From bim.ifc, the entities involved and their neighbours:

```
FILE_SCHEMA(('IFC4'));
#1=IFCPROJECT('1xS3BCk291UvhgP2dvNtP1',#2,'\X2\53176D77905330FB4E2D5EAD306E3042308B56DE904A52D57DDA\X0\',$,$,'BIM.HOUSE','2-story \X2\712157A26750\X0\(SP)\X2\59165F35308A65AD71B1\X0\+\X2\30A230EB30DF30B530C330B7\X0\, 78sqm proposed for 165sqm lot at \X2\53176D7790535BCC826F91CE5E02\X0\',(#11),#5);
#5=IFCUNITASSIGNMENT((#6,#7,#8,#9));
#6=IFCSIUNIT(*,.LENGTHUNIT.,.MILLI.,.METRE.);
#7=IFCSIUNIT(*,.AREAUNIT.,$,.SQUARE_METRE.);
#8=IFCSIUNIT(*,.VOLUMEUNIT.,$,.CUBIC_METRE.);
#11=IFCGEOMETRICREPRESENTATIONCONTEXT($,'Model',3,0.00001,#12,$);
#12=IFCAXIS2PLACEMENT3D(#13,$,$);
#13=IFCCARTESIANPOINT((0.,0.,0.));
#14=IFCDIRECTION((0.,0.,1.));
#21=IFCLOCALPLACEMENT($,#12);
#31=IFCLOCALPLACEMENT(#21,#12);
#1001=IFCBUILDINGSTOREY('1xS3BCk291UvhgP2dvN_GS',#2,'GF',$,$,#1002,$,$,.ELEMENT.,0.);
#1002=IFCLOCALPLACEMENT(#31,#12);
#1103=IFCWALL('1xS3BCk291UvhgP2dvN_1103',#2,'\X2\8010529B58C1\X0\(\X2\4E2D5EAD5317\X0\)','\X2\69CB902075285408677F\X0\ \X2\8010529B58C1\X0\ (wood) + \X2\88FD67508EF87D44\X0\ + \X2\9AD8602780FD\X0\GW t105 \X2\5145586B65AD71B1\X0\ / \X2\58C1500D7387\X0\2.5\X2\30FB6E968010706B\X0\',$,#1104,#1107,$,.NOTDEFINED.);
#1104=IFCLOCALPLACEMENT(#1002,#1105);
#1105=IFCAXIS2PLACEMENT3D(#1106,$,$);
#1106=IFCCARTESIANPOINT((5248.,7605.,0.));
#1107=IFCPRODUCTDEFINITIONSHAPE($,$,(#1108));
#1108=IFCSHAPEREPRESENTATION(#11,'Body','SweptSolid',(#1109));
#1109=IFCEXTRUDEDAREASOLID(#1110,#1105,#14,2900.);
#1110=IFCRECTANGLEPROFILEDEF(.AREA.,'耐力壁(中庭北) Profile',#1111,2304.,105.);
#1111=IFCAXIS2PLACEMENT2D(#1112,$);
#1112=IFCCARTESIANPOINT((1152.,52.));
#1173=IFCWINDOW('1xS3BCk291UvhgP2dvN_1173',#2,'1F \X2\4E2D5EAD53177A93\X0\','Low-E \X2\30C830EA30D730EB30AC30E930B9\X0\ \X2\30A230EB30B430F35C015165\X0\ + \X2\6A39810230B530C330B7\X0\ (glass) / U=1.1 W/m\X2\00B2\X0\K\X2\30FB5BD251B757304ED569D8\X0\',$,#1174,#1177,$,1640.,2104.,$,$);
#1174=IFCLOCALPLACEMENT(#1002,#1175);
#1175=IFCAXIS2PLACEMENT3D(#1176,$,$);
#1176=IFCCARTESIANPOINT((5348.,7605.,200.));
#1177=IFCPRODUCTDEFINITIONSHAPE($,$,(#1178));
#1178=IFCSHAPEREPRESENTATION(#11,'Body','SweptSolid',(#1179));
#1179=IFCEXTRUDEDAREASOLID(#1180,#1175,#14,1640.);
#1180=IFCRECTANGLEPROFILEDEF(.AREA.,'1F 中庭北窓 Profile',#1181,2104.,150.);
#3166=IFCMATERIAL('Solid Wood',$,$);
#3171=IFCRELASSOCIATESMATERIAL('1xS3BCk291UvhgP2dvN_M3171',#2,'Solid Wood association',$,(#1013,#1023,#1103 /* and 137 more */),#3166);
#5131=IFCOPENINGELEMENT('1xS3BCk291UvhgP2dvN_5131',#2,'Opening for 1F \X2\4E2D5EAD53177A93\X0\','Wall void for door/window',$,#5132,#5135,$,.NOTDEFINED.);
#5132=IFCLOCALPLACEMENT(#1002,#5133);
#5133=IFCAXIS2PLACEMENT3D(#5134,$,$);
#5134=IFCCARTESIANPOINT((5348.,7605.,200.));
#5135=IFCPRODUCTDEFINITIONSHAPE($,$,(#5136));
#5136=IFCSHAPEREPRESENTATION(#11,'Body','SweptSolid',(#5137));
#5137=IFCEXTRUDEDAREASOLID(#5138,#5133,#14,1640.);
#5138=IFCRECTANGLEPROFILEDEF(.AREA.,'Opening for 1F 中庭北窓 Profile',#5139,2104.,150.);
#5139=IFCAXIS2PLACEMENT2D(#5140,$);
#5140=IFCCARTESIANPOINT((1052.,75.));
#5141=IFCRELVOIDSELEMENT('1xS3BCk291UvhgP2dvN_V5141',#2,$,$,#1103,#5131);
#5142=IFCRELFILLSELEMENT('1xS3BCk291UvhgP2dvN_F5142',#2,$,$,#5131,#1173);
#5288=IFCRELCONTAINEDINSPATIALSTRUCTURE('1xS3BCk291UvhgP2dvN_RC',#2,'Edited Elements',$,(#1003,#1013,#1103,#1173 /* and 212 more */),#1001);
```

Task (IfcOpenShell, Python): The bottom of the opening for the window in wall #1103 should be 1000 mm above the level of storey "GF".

```python
import numpy as np
import ifcopenshell
import ifcopenshell.api.geometry
import ifcopenshell.geom
import ifcopenshell.util.element
import ifcopenshell.util.placement
import ifcopenshell.util.shape
import ifcopenshell.util.unit

model = ifcopenshell.open("bim.ifc")
unit_scale = ifcopenshell.util.unit.calculate_unit_scale(model)

window = model.by_guid("1xS3BCk291UvhgP2dvN_1173")
opening = window.FillsVoids[0].RelatingOpeningElement
storey = ifcopenshell.util.element.get_container(window, ifc_class="IfcBuildingStorey")
level = ifcopenshell.util.placement.get_local_placement(storey.ObjectPlacement)[2, 3]

# The opening's origin need not be at the sill, so measure its lowest point.
shape = ifcopenshell.geom.create_shape(ifcopenshell.geom.settings(), opening)
bottom = ifcopenshell.util.shape.get_shape_bottom_elevation(shape, shape.geometry) / unit_scale
dz = level + 1 / unit_scale - bottom

shift = np.array([0.0, 0.0, dz])
# The window is not placed relative to its opening, so move both.
for product in (opening, window):
    matrix = ifcopenshell.util.placement.get_local_placement(product.ObjectPlacement)
    matrix[:3, 3] += shift
    ifcopenshell.api.geometry.edit_object_placement(model, product=product, matrix=matrix, is_si=False)

print(f"moved by {dz * unit_scale:+.3f} m")

model.write("bim-out.ifc")
```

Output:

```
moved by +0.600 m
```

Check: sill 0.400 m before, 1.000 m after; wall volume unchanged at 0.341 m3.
